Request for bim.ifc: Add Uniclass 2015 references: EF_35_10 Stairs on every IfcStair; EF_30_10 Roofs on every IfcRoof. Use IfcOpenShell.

First a look at what the model holds.

```python
import ifcopenshell

model = ifcopenshell.open("bim.ifc")
print(model.schema)
print("classifications:", [c.Name for c in model.by_type("IfcClassification")])
for ifc_class in ("IfcDoor", "IfcRoof", "IfcStair", "IfcWall", "IfcWindow"):
    print(ifc_class, len(model.by_type(ifc_class)))
```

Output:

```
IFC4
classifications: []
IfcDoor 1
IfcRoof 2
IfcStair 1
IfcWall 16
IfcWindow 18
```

```python
import ifcopenshell
import ifcopenshell.api.classification

model = ifcopenshell.open("bim.ifc")

system = ifcopenshell.api.classification.add_classification(model, classification="Uniclass 2015")

codes = {
    "IfcStair": ("EF_35_10", "Stairs"),
    "IfcRoof": ("EF_30_10", "Roofs"),
}
for ifc_class, (code, name) in codes.items():
    products = model.by_type(ifc_class)
    ifcopenshell.api.classification.add_reference(
        model, products=products, classification=system, identification=code, name=name
    )
    print(code, len(products))

model.write("bim_v2.ifc")
```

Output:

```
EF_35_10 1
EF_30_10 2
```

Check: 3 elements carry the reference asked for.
